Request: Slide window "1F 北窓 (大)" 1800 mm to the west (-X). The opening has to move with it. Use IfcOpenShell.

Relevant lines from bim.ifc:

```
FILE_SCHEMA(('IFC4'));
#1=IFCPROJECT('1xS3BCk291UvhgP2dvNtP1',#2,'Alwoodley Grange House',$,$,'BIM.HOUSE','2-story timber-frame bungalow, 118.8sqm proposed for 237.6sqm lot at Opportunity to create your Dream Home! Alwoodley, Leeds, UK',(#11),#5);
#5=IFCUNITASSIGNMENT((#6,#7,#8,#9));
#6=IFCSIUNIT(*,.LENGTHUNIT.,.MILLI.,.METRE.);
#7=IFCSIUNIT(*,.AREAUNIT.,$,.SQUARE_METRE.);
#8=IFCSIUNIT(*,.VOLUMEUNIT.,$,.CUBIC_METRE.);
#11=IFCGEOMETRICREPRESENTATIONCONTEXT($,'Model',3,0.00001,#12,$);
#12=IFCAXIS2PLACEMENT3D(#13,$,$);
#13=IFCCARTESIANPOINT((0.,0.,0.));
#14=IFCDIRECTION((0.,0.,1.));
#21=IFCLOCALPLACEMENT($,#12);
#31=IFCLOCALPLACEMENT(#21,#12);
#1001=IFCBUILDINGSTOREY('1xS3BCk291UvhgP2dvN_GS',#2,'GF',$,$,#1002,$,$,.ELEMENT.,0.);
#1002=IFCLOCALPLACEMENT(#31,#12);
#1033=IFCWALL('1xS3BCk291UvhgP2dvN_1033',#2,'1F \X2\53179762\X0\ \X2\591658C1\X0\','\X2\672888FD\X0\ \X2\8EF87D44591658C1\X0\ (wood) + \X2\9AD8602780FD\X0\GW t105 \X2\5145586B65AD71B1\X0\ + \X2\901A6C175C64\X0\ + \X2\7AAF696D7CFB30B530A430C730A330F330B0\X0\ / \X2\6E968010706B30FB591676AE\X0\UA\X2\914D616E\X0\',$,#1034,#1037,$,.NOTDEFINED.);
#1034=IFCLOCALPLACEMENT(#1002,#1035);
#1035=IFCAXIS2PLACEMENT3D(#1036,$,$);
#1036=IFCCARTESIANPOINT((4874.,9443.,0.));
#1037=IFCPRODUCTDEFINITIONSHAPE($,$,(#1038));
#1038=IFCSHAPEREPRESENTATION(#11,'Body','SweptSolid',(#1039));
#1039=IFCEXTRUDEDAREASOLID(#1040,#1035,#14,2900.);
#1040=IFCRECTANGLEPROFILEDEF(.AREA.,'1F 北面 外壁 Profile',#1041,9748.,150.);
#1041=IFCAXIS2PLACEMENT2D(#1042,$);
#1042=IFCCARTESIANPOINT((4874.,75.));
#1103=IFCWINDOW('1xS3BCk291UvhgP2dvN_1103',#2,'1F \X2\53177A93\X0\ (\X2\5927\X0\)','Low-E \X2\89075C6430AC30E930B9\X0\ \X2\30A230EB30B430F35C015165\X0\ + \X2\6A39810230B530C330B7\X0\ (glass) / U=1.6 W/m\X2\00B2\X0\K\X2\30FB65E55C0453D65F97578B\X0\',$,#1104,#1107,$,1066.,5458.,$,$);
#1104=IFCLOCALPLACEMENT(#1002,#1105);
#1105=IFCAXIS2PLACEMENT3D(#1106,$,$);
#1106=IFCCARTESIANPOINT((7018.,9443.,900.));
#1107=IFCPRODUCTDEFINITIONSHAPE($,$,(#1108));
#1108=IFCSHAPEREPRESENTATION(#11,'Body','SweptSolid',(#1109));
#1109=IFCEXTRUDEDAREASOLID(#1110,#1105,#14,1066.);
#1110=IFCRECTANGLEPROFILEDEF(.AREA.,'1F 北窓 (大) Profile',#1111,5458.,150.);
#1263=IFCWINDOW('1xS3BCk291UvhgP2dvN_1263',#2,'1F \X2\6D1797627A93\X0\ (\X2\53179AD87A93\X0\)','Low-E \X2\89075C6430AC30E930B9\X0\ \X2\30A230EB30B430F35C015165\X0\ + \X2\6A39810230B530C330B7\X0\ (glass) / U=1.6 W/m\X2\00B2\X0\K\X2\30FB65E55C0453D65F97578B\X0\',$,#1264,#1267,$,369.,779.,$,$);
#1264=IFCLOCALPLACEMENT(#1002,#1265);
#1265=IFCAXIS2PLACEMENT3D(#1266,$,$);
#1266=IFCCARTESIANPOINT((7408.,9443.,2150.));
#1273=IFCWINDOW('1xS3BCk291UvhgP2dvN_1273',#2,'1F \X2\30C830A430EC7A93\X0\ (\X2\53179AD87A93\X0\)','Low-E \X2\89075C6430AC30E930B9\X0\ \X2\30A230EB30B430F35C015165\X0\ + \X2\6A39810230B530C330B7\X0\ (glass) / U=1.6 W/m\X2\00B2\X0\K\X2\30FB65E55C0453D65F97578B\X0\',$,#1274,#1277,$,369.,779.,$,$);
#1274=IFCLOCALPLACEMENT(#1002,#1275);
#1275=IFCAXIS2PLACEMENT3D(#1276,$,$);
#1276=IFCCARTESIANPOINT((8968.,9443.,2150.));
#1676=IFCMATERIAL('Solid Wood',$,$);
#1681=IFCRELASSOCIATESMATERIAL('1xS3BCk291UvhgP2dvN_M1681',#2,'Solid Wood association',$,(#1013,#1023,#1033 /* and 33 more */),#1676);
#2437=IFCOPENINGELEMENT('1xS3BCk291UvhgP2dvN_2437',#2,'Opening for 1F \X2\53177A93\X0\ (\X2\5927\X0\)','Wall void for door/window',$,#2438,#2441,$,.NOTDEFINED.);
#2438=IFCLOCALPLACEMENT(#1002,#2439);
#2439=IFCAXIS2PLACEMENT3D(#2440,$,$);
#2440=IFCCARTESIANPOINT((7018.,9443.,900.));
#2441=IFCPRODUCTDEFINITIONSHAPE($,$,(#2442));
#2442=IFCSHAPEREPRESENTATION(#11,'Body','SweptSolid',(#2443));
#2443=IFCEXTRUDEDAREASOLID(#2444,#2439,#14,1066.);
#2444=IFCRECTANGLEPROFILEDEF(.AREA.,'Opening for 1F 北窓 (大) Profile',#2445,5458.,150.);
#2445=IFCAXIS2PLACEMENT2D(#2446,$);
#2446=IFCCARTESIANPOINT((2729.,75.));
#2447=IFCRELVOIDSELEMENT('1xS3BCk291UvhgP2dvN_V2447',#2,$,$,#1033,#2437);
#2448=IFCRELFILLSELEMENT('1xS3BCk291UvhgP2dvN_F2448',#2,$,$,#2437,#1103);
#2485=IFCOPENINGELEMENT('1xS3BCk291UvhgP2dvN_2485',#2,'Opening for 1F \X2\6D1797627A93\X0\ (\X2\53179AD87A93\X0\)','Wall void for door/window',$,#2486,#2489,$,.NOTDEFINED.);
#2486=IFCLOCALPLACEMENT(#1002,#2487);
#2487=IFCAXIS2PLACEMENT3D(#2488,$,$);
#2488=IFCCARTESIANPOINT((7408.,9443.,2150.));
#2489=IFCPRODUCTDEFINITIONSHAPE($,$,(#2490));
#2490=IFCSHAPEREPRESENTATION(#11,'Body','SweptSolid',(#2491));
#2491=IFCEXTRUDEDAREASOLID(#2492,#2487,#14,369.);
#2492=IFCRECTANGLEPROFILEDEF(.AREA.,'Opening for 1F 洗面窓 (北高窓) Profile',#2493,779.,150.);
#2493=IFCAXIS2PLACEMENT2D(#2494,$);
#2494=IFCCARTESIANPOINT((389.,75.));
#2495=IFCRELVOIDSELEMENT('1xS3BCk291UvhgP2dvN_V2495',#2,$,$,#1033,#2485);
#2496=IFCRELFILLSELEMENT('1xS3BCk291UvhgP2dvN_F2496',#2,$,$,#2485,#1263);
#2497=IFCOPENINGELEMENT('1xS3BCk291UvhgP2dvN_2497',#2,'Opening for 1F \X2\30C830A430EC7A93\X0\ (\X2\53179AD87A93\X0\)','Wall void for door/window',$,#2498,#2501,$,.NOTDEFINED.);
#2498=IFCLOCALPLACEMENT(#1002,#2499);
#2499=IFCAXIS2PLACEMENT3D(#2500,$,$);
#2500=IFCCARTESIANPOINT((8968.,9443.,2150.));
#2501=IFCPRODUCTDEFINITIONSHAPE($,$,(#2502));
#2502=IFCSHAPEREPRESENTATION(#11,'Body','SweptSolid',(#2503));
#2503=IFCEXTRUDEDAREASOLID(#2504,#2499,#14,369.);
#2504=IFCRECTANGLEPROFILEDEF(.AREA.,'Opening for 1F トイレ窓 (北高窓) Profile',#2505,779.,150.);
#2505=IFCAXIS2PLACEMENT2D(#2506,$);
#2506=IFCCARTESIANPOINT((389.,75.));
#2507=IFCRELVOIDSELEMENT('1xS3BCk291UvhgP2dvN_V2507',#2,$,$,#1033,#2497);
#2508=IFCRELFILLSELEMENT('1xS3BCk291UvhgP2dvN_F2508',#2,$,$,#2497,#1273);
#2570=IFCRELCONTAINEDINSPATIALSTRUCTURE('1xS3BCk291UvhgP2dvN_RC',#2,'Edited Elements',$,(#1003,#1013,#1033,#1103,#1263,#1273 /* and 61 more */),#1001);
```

```python
import ifcopenshell
import ifcopenshell.api.geometry
import ifcopenshell.util.placement
import ifcopenshell.util.unit

model = ifcopenshell.open("bim.ifc")
unit_scale = ifcopenshell.util.unit.calculate_unit_scale(model)

window = model.by_guid("1xS3BCk291UvhgP2dvN_1103")
opening = window.FillsVoids[0].RelatingOpeningElement
wall = opening.VoidsElements[0].RelatingBuildingElement

wall_matrix = ifcopenshell.util.placement.get_local_placement(wall.ObjectPlacement)
shift = wall_matrix[:3, 0] * -1.8 / unit_scale
before = ifcopenshell.util.placement.get_local_placement(window.ObjectPlacement)[:3, 3].copy()

# The window is not placed relative to its opening, so move both.
for product in (opening, window):
    matrix = ifcopenshell.util.placement.get_local_placement(product.ObjectPlacement)
    matrix[:3, 3] += shift
    ifcopenshell.api.geometry.edit_object_placement(model, product=product, matrix=matrix, is_si=False)

after = ifcopenshell.util.placement.get_local_placement(window.ObjectPlacement)[:3, 3]
print("window moved by", (after - before).round(3) + 0.0)

model.write("bim_v2.ifc")
```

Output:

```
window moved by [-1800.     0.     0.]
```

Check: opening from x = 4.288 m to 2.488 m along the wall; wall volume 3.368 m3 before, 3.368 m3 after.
